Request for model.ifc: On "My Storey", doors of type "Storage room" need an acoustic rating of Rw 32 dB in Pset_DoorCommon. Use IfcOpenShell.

First a look at what the model holds.

```python
import ifcopenshell
import ifcopenshell.util.element

model = ifcopenshell.open("model.ifc")
print(model.schema)
storey = next(s for s in model.by_type("IfcBuildingStorey") if s.Name == "My Storey")
doors = [e for e in ifcopenshell.util.element.get_decomposition(storey) if e.is_a("IfcDoor")]
seen = {}
for e in doors:
    element_type = ifcopenshell.util.element.get_type(e)
    key = (element_type.Name if element_type != e and element_type else None, ifcopenshell.util.element.get_pset(e, "Pset_DoorCommon", "AcousticRating"))
    seen[key] = seen.get(key, 0) + 1
for (name, value), count in sorted(seen.items(), key=str):
    print(count, "x", name, "|", value)
```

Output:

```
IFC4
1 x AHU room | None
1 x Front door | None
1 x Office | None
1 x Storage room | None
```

```python
import ifcopenshell
import ifcopenshell.api.pset
import ifcopenshell.util.element

model = ifcopenshell.open("model.ifc")

storey = next(s for s in model.by_type("IfcBuildingStorey") if s.Name == "My Storey")
doors = [e for e in ifcopenshell.util.element.get_decomposition(storey) if e.is_a("IfcDoor")]

count = 0
for e in doors:
    element_type = ifcopenshell.util.element.get_type(e)
    if element_type in (None, e) or element_type.Name != "Storage room":
        continue
    # add_pset returns the element's existing set when there is one.
    pset = ifcopenshell.api.pset.add_pset(model, product=e, name="Pset_DoorCommon")
    ifcopenshell.api.pset.edit_pset(model, pset=pset, properties={"AcousticRating": "Rw 32 dB"})
    count += 1

print(count, "doors updated")

model.write("model_rev.ifc")
```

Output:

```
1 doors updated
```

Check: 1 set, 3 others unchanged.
